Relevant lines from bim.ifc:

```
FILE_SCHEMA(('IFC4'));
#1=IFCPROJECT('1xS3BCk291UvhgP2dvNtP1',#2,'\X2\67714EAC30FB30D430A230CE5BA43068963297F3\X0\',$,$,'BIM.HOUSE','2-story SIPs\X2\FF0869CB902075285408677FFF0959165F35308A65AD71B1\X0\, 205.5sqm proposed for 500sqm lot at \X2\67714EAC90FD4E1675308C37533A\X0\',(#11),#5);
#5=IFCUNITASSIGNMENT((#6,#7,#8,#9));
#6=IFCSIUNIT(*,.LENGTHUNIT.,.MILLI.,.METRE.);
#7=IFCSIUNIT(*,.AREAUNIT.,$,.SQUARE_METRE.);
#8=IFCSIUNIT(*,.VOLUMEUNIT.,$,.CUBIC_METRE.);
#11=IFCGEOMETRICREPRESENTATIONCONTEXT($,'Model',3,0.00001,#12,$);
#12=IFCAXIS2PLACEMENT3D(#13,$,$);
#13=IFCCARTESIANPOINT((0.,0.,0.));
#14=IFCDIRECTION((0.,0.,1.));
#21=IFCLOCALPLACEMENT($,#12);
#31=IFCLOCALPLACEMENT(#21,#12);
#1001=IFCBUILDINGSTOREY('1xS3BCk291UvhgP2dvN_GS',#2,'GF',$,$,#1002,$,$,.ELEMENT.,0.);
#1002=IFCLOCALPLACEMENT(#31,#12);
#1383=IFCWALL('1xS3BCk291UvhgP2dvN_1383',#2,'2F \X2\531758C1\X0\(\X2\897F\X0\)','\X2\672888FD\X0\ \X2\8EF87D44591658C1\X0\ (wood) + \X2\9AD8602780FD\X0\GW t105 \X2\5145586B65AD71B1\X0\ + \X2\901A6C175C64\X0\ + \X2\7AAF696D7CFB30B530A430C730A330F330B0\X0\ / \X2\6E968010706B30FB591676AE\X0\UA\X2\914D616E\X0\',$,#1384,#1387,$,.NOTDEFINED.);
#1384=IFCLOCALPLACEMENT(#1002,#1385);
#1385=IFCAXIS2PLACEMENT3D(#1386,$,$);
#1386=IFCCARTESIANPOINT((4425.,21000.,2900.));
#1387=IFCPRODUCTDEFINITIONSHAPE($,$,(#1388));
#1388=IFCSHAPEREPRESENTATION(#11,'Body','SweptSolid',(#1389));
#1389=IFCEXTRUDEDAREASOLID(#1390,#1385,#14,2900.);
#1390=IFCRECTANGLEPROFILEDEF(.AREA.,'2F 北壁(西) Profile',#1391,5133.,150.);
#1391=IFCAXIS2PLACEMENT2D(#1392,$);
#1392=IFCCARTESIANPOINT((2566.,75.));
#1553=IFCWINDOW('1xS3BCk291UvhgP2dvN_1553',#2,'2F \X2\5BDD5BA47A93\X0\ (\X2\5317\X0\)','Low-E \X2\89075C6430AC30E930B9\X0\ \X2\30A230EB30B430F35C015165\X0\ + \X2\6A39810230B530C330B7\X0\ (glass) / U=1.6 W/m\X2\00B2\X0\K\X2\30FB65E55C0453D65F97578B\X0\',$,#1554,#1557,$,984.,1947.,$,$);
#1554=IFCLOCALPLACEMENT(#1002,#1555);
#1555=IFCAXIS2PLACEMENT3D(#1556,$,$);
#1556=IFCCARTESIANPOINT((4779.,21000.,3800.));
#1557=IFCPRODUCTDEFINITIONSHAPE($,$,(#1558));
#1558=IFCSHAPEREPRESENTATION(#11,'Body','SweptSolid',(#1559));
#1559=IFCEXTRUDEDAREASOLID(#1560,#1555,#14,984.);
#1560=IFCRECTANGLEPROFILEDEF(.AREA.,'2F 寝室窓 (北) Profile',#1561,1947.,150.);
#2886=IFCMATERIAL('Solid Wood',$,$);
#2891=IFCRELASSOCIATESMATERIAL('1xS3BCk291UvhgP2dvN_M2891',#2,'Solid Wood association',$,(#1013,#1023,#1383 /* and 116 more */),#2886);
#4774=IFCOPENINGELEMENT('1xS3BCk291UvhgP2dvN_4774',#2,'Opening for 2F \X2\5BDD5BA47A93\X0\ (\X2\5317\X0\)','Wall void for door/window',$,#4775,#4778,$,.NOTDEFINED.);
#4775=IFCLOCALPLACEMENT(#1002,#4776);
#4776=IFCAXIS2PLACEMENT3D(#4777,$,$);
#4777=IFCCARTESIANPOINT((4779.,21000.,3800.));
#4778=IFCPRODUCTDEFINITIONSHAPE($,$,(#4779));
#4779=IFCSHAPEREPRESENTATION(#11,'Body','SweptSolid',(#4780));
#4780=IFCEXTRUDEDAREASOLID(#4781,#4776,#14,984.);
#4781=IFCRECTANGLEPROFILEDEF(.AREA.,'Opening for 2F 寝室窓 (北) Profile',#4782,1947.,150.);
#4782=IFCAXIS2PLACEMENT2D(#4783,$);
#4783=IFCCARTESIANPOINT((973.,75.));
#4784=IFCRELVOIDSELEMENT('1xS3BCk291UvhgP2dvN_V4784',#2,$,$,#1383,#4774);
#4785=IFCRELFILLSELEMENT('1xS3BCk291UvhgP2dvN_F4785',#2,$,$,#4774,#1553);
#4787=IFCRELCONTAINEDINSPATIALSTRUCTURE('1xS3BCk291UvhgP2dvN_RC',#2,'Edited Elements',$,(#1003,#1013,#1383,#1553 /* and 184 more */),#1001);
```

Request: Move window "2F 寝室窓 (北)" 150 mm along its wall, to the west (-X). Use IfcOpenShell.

```python
import ifcopenshell
import ifcopenshell.api.geometry
import ifcopenshell.util.placement

model = ifcopenshell.open("bim.ifc")

window = model.by_guid("1xS3BCk291UvhgP2dvN_1553")
opening = window.FillsVoids[0].RelatingOpeningElement
wall = opening.VoidsElements[0].RelatingBuildingElement

wall_matrix = ifcopenshell.util.placement.get_local_placement(wall.ObjectPlacement)
shift = wall_matrix[:3, 0] * -150.0
before = ifcopenshell.util.placement.get_local_placement(window.ObjectPlacement)[:3, 3].copy()

# The window is not placed relative to its opening, so move both.
for product in (opening, window):
    matrix = ifcopenshell.util.placement.get_local_placement(product.ObjectPlacement)
    matrix[:3, 3] += shift
    ifcopenshell.api.geometry.edit_object_placement(model, product=product, matrix=matrix, is_si=False)

after = ifcopenshell.util.placement.get_local_placement(window.ObjectPlacement)[:3, 3]
print("window moved by", (after - before).round(3) + 0.0)

model.write("bim_v2.ifc")
```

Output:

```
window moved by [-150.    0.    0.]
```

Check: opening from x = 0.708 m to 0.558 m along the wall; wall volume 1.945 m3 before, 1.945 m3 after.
